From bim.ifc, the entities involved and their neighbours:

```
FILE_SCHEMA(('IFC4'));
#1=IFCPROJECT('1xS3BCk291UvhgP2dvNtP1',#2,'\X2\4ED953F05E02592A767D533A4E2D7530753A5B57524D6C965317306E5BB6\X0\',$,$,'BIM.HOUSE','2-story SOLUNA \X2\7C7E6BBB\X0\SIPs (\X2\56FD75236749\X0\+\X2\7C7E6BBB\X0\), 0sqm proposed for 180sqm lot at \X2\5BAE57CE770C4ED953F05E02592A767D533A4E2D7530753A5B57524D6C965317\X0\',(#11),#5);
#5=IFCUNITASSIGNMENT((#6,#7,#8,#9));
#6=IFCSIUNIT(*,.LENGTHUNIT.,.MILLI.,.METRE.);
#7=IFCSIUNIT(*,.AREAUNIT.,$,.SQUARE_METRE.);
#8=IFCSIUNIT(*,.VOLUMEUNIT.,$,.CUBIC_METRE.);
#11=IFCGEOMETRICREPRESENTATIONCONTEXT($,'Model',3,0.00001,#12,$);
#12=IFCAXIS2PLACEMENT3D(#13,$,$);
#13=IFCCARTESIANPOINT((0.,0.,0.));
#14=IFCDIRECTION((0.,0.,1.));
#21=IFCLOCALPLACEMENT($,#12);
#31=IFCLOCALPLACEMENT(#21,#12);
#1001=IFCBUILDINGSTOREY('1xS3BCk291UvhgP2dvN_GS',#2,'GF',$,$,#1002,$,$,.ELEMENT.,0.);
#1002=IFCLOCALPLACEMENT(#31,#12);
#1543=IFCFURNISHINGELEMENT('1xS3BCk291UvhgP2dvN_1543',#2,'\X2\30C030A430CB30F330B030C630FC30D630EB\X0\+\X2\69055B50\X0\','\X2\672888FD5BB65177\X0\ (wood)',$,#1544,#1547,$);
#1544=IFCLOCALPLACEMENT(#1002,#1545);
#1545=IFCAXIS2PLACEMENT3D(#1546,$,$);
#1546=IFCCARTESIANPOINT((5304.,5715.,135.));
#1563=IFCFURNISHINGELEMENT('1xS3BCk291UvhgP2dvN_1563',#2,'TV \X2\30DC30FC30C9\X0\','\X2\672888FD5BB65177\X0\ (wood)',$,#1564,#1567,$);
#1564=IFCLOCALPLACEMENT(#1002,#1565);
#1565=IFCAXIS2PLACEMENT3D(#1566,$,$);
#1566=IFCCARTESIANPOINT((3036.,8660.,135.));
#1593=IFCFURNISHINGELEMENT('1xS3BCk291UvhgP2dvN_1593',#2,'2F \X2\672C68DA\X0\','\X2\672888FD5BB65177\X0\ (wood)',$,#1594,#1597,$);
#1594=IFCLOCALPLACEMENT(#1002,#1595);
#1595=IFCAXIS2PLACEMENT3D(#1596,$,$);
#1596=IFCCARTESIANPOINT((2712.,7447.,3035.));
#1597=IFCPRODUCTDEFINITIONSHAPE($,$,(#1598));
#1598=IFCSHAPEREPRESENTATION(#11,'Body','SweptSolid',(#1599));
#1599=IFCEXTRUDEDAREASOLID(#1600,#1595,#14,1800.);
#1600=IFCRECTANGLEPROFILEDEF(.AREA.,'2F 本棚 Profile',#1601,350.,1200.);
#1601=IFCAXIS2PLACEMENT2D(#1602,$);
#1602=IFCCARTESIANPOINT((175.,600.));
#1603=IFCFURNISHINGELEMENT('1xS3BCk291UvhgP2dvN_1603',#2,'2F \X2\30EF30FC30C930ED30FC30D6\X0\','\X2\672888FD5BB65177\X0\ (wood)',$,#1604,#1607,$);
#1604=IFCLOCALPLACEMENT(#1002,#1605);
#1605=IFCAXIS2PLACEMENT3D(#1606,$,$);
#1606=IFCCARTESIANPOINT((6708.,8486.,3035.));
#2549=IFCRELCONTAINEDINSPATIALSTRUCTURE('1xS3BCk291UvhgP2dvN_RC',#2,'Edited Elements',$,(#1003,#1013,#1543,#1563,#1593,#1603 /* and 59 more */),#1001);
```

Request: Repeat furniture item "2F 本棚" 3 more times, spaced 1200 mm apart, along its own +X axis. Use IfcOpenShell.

```python
import ifcopenshell
import ifcopenshell.api.geometry
import ifcopenshell.api.root
import ifcopenshell.util.element
import ifcopenshell.util.placement

model = ifcopenshell.open("bim.ifc")


def reuse_history(source, copy):
    """copy_class also copies each property set's owner history, people and application; keep the originals."""
    for rel in copy.IsDefinedBy:
        if rel.is_a("IfcRelDefinesByProperties") and (history := rel.RelatingPropertyDefinition.OwnerHistory):
            rel.RelatingPropertyDefinition.OwnerHistory = source.OwnerHistory
            ifcopenshell.util.element.remove_deep2(model, history)


source = model.by_guid("1xS3BCk291UvhgP2dvN_1593")
base = ifcopenshell.util.placement.get_local_placement(source.ObjectPlacement)
step = base[:3, 0] * 1200.0

for i in range(1, 4):
    copy = ifcopenshell.api.root.copy_class(model, product=source)
    copy.Representation = ifcopenshell.util.element.copy_deep(
        model, source.Representation, exclude=["IfcGeometricRepresentationContext", "IfcRepresentationMap"]
    )
    reuse_history(source, copy)
    matrix = base.copy()
    matrix[:3, 3] += i * step
    print("added at", matrix[:3, 3].round(3) + 0.0)
    ifcopenshell.api.geometry.edit_object_placement(model, product=copy, matrix=matrix, is_si=False)

model.write("bim_updated.ifc")
```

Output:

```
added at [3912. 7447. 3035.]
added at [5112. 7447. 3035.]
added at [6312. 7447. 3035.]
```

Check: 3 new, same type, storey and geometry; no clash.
